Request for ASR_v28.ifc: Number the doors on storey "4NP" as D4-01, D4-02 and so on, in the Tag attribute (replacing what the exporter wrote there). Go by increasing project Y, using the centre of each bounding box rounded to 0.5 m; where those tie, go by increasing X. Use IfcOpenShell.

First a look at what the model holds.

```python
import ifcopenshell
import ifcopenshell.util.element
import ifcopenshell.util.placement

model = ifcopenshell.open("ASR_v28.ifc")
print(model.schema)
storey = next(s for s in model.by_type("IfcBuildingStorey") if s.Name == "4NP")
doors = [e for e in ifcopenshell.util.element.get_decomposition(storey) if e.is_a("IfcDoor")]
for e in sorted(doors, key=lambda e: e.id()):
    origin = ifcopenshell.util.placement.get_local_placement(e.ObjectPlacement)[:3, 3]
    print(e.id(), e.Tag, e.Name, origin.round(2) + 0.0, sep=" | ")
```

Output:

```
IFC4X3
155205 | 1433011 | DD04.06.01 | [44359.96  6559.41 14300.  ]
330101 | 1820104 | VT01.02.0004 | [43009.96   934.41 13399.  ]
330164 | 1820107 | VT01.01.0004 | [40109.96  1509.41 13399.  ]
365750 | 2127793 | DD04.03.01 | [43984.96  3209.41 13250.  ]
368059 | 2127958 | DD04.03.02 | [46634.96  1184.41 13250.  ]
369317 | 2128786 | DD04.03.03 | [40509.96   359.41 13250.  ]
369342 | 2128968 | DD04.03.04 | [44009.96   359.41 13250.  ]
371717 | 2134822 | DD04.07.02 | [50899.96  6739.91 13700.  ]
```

```python
import ifcopenshell
import ifcopenshell.geom
import ifcopenshell.util.element
import ifcopenshell.util.shape

model = ifcopenshell.open("ASR_v28.ifc")
settings = ifcopenshell.geom.settings()
settings.set("use-world-coords", True)


def centre(element):
    shape = ifcopenshell.geom.create_shape(settings, element)
    return ifcopenshell.util.shape.get_bbox_centroid(shape.geometry)


storey = next(s for s in model.by_type("IfcBuildingStorey") if s.Name == "4NP")
doors = [e for e in ifcopenshell.util.element.get_decomposition(storey) if e.is_a("IfcDoor")]

# Insertion points can sit at a corner or the storey origin, so sort by the geometry (in metres).
centres = {e: centre(e) for e in doors}
doors.sort(key=lambda e: (round(centres[e][1] / 0.5), centres[e][0]))

for i, e in enumerate(doors, start=1):
    number = f"D4-{i:02d}"
    e.Tag = number
    print(e.id(), number)

model.write("ASR_v28_rev.ifc")
```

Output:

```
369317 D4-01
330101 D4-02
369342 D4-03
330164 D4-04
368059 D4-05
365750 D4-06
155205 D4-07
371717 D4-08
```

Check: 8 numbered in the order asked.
